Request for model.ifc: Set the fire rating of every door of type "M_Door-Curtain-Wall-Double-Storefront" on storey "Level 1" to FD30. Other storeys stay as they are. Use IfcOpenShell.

First a look at what the model holds.

```python
import ifcopenshell
import ifcopenshell.util.element

model = ifcopenshell.open("model.ifc")
print(model.schema)
storey = next(s for s in model.by_type("IfcBuildingStorey") if s.Name == "Level 1")
doors = [e for e in ifcopenshell.util.element.get_decomposition(storey) if e.is_a("IfcDoor")]
seen = {}
for e in doors:
    element_type = ifcopenshell.util.element.get_type(e)
    key = (element_type.Name if element_type != e and element_type else None, ifcopenshell.util.element.get_pset(e, "Pset_DoorCommon", "FireRating"))
    seen[key] = seen.get(key, 0) + 1
for (name, value), count in sorted(seen.items(), key=str):
    print(count, "x", name, "|", value)
```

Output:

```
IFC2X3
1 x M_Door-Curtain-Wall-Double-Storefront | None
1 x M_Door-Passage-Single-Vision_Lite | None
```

```python
import ifcopenshell
import ifcopenshell.api.pset
import ifcopenshell.util.element

model = ifcopenshell.open("model.ifc")

storey = next(s for s in model.by_type("IfcBuildingStorey") if s.Name == "Level 1")
doors = [e for e in ifcopenshell.util.element.get_decomposition(storey) if e.is_a("IfcDoor")]

count = 0
for e in doors:
    element_type = ifcopenshell.util.element.get_type(e)
    if element_type in (None, e) or element_type.Name != "M_Door-Curtain-Wall-Double-Storefront":
        continue
    # add_pset returns the element's existing set when there is one.
    pset = ifcopenshell.api.pset.add_pset(model, product=e, name="Pset_DoorCommon")
    ifcopenshell.api.pset.edit_pset(model, pset=pset, properties={"FireRating": "FD30"})
    count += 1

print(count, "doors updated")

model.write("model_v2.ifc")
```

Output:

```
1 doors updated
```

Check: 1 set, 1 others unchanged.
